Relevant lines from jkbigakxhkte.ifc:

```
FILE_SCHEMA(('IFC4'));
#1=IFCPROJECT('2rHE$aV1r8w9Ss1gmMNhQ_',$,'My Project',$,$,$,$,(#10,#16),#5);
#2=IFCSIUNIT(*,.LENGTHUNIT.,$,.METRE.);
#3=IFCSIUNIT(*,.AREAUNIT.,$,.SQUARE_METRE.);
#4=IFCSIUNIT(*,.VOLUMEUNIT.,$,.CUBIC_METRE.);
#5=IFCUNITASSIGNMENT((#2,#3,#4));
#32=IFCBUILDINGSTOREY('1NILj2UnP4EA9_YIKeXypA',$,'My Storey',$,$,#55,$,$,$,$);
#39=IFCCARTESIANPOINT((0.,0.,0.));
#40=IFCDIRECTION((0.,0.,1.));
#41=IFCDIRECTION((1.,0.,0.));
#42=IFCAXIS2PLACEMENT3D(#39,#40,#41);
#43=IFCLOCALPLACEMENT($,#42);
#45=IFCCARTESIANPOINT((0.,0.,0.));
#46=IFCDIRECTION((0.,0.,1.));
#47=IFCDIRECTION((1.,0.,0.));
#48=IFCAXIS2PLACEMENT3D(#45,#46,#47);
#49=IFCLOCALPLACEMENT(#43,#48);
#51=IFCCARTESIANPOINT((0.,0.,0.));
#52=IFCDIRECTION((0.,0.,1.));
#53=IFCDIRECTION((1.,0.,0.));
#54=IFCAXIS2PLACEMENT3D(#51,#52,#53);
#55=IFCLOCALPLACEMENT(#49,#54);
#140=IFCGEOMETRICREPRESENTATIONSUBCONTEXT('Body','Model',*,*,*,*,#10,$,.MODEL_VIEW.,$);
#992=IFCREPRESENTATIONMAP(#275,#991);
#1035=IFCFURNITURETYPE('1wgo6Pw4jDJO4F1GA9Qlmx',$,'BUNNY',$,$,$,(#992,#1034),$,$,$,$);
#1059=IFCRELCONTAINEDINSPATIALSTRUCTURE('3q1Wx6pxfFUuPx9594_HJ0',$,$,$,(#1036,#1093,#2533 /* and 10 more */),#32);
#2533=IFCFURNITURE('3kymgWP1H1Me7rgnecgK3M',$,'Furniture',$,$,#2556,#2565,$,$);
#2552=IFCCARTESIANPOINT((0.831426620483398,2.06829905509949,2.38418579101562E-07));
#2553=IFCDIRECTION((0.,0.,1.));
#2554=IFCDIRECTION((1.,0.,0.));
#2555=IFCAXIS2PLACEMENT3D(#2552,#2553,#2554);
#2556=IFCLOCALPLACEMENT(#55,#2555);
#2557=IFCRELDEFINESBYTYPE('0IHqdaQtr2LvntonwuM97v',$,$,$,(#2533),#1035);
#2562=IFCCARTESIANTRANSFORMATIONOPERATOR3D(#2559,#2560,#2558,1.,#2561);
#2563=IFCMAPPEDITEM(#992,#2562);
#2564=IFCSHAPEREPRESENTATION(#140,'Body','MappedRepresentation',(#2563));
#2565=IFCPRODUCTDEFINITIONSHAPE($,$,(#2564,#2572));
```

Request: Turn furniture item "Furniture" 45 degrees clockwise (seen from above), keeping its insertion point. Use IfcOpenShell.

```python
import ifcopenshell
import ifcopenshell.api.geometry
import ifcopenshell.util.placement

model = ifcopenshell.open("jkbigakxhkte.ifc")

item = model.by_guid("3kymgWP1H1Me7rgnecgK3M")
matrix = ifcopenshell.util.placement.get_local_placement(item.ObjectPlacement)
matrix = matrix @ ifcopenshell.util.placement.rotation(-45, "Z")
ifcopenshell.api.geometry.edit_object_placement(model, product=item, matrix=matrix, is_si=False)

print(ifcopenshell.util.placement.get_local_placement(item.ObjectPlacement).round(3) + 0.0)

model.write("jkbigakxhkte_v2.ifc")
```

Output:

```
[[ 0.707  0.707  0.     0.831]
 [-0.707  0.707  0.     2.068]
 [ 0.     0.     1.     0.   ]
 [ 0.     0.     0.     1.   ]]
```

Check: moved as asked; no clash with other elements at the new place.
